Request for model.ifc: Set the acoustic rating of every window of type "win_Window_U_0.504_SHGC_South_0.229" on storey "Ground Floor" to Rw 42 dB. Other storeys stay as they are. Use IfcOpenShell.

First a look at what the model holds.

```python
import ifcopenshell
import ifcopenshell.util.element

model = ifcopenshell.open("model.ifc")
print(model.schema)
storey = next(s for s in model.by_type("IfcBuildingStorey") if s.Name == "Ground Floor")
windows = [e for e in ifcopenshell.util.element.get_decomposition(storey) if e.is_a("IfcWindow")]
seen = {}
for e in windows:
    element_type = ifcopenshell.util.element.get_type(e)
    key = (element_type.Name if element_type != e and element_type else None, ifcopenshell.util.element.get_pset(e, "Pset_WindowCommon", "AcousticRating"))
    seen[key] = seen.get(key, 0) + 1
for (name, value), count in sorted(seen.items(), key=str):
    print(count, "x", name, "|", value)
```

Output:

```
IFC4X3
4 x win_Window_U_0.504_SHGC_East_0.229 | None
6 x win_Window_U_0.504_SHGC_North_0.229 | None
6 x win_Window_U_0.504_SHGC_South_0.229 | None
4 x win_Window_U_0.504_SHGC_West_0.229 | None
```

```python
import ifcopenshell
import ifcopenshell.api.pset
import ifcopenshell.util.element

model = ifcopenshell.open("model.ifc")

storey = next(s for s in model.by_type("IfcBuildingStorey") if s.Name == "Ground Floor")
windows = [e for e in ifcopenshell.util.element.get_decomposition(storey) if e.is_a("IfcWindow")]

count = 0
for e in windows:
    element_type = ifcopenshell.util.element.get_type(e)
    if element_type in (None, e) or element_type.Name != "win_Window_U_0.504_SHGC_South_0.229":
        continue
    # add_pset returns the element's existing set when there is one.
    pset = ifcopenshell.api.pset.add_pset(model, product=e, name="Pset_WindowCommon")
    ifcopenshell.api.pset.edit_pset(model, pset=pset, properties={"AcousticRating": "Rw 42 dB"})
    count += 1

print(count, "windows updated")

model.write("model-out.ifc")
```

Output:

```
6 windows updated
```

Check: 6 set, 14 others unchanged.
